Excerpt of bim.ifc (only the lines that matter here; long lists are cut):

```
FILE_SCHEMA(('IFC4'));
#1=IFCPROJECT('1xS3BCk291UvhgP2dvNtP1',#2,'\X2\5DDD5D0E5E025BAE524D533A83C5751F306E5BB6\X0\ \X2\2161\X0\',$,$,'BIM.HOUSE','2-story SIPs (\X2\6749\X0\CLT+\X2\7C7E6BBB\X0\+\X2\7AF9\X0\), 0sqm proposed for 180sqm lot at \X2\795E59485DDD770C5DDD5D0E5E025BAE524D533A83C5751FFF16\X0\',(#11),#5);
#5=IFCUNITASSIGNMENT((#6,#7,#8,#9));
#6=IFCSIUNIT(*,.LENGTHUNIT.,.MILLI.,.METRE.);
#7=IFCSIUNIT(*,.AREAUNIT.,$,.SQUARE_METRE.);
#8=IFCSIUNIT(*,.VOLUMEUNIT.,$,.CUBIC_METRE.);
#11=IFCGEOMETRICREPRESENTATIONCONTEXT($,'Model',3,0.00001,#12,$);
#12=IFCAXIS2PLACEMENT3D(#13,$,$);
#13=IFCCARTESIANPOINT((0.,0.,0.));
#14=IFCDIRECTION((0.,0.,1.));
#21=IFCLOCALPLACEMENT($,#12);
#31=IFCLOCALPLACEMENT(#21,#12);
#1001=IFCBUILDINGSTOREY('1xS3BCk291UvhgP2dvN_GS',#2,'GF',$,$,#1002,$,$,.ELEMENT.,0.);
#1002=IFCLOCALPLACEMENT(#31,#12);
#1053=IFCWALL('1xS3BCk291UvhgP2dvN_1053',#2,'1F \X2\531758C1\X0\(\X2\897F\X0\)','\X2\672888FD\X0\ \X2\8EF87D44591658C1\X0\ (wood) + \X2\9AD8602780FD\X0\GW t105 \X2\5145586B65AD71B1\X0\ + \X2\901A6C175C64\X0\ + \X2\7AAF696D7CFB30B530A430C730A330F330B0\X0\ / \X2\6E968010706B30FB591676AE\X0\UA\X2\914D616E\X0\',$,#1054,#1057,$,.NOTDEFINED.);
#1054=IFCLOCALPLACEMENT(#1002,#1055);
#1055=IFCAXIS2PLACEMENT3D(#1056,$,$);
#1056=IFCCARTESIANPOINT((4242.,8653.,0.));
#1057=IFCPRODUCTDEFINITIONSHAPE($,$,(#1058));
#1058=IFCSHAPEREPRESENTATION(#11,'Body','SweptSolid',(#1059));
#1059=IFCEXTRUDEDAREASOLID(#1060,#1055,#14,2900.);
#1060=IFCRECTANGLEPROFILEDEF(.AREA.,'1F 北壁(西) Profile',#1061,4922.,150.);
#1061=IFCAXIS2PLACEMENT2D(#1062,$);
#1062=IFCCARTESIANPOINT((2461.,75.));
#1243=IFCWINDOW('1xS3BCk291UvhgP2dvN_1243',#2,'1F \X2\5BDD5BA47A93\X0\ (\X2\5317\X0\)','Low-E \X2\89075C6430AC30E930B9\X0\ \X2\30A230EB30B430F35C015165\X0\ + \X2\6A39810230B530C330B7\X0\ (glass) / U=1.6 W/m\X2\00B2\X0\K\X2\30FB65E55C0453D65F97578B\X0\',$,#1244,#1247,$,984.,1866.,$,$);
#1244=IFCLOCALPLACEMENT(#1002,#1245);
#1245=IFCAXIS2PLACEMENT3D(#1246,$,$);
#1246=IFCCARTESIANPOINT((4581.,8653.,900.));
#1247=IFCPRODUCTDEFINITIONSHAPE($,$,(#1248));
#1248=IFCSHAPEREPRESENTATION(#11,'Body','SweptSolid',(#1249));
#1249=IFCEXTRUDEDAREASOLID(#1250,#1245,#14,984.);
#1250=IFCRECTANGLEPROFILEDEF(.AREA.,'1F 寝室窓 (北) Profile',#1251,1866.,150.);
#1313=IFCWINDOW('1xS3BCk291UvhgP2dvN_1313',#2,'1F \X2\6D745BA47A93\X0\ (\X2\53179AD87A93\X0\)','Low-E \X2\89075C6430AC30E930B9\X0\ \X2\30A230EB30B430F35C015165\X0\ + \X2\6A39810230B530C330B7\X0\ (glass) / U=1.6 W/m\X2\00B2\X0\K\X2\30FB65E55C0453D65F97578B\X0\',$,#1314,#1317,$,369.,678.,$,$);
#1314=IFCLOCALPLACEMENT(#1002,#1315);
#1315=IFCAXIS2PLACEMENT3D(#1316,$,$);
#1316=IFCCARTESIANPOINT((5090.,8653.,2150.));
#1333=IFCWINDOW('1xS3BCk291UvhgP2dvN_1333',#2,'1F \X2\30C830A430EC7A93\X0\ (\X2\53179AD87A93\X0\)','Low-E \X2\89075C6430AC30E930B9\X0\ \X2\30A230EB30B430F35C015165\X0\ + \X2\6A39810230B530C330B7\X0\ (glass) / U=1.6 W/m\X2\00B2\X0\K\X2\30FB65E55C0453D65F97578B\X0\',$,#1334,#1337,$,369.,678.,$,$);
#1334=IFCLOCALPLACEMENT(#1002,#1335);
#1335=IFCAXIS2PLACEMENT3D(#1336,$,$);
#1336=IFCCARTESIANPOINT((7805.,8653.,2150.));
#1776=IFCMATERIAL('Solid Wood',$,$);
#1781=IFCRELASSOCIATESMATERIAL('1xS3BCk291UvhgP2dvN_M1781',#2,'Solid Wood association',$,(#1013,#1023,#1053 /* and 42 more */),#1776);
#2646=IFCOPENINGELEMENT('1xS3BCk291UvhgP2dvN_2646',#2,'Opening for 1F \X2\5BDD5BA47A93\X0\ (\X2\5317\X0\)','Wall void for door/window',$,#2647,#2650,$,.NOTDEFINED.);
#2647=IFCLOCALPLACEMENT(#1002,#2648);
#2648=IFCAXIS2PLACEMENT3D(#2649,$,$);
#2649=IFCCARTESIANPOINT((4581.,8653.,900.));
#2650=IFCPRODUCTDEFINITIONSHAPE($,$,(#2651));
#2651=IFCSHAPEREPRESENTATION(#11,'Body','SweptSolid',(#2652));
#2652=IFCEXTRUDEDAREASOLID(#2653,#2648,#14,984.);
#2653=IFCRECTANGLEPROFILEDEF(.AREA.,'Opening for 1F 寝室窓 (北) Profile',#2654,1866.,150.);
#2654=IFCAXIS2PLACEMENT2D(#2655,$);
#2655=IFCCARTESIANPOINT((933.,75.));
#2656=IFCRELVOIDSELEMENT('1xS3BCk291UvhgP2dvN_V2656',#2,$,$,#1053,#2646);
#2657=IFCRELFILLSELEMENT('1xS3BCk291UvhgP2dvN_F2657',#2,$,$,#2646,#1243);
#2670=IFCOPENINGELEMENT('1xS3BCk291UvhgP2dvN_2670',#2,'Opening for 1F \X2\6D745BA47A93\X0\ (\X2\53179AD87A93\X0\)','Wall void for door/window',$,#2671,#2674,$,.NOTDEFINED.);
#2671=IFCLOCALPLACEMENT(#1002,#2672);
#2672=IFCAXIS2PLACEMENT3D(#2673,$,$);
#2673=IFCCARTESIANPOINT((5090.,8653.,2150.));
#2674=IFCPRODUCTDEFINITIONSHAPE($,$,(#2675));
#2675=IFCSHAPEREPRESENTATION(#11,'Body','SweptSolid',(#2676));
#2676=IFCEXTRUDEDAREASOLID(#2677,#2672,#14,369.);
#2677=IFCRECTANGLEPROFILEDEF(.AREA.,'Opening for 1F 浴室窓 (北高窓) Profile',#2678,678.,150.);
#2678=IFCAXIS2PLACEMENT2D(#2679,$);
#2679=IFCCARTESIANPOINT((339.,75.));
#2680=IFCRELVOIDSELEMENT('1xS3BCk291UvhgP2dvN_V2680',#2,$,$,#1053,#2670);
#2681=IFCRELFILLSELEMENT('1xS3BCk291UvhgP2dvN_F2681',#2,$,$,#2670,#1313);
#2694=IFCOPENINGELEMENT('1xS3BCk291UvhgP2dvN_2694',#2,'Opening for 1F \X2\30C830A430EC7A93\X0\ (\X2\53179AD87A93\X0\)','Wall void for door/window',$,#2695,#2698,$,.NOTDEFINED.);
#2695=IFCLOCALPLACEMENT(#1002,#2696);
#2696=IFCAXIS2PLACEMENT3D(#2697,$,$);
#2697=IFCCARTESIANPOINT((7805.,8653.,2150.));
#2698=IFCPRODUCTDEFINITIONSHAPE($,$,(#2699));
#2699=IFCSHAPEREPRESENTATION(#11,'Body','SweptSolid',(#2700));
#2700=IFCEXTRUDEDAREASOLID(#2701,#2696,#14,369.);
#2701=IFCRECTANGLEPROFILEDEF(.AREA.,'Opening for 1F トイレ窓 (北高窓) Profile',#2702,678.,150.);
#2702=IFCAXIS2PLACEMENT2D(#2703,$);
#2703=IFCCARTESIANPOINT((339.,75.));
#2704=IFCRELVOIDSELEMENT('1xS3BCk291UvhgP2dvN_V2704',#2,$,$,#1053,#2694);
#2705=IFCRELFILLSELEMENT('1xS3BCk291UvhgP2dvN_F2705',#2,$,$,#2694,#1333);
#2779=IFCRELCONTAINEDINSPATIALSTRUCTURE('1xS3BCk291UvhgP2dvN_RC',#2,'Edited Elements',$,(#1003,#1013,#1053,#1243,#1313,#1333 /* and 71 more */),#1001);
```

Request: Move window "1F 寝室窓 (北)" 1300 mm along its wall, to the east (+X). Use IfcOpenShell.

```python
import ifcopenshell
import ifcopenshell.api.geometry
import ifcopenshell.util.placement
import ifcopenshell.util.unit

model = ifcopenshell.open("bim.ifc")
unit_scale = ifcopenshell.util.unit.calculate_unit_scale(model)

window = model.by_id(1243)
opening = window.FillsVoids[0].RelatingOpeningElement
wall = opening.VoidsElements[0].RelatingBuildingElement

wall_matrix = ifcopenshell.util.placement.get_local_placement(wall.ObjectPlacement)
shift = wall_matrix[:3, 0] * 1.3 / unit_scale
before = ifcopenshell.util.placement.get_local_placement(window.ObjectPlacement)[:3, 3].copy()

# The window is not placed relative to its opening, so move both.
for product in (opening, window):
    matrix = ifcopenshell.util.placement.get_local_placement(product.ObjectPlacement)
    matrix[:3, 3] += shift
    ifcopenshell.api.geometry.edit_object_placement(model, product=product, matrix=matrix, is_si=False)

after = ifcopenshell.util.placement.get_local_placement(window.ObjectPlacement)[:3, 3]
print("window moved by", (after - before).round(3) + 0.0)

model.write("bim-out.ifc")
```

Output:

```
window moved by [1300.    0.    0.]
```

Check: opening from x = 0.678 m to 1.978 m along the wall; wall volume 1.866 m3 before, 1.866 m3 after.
